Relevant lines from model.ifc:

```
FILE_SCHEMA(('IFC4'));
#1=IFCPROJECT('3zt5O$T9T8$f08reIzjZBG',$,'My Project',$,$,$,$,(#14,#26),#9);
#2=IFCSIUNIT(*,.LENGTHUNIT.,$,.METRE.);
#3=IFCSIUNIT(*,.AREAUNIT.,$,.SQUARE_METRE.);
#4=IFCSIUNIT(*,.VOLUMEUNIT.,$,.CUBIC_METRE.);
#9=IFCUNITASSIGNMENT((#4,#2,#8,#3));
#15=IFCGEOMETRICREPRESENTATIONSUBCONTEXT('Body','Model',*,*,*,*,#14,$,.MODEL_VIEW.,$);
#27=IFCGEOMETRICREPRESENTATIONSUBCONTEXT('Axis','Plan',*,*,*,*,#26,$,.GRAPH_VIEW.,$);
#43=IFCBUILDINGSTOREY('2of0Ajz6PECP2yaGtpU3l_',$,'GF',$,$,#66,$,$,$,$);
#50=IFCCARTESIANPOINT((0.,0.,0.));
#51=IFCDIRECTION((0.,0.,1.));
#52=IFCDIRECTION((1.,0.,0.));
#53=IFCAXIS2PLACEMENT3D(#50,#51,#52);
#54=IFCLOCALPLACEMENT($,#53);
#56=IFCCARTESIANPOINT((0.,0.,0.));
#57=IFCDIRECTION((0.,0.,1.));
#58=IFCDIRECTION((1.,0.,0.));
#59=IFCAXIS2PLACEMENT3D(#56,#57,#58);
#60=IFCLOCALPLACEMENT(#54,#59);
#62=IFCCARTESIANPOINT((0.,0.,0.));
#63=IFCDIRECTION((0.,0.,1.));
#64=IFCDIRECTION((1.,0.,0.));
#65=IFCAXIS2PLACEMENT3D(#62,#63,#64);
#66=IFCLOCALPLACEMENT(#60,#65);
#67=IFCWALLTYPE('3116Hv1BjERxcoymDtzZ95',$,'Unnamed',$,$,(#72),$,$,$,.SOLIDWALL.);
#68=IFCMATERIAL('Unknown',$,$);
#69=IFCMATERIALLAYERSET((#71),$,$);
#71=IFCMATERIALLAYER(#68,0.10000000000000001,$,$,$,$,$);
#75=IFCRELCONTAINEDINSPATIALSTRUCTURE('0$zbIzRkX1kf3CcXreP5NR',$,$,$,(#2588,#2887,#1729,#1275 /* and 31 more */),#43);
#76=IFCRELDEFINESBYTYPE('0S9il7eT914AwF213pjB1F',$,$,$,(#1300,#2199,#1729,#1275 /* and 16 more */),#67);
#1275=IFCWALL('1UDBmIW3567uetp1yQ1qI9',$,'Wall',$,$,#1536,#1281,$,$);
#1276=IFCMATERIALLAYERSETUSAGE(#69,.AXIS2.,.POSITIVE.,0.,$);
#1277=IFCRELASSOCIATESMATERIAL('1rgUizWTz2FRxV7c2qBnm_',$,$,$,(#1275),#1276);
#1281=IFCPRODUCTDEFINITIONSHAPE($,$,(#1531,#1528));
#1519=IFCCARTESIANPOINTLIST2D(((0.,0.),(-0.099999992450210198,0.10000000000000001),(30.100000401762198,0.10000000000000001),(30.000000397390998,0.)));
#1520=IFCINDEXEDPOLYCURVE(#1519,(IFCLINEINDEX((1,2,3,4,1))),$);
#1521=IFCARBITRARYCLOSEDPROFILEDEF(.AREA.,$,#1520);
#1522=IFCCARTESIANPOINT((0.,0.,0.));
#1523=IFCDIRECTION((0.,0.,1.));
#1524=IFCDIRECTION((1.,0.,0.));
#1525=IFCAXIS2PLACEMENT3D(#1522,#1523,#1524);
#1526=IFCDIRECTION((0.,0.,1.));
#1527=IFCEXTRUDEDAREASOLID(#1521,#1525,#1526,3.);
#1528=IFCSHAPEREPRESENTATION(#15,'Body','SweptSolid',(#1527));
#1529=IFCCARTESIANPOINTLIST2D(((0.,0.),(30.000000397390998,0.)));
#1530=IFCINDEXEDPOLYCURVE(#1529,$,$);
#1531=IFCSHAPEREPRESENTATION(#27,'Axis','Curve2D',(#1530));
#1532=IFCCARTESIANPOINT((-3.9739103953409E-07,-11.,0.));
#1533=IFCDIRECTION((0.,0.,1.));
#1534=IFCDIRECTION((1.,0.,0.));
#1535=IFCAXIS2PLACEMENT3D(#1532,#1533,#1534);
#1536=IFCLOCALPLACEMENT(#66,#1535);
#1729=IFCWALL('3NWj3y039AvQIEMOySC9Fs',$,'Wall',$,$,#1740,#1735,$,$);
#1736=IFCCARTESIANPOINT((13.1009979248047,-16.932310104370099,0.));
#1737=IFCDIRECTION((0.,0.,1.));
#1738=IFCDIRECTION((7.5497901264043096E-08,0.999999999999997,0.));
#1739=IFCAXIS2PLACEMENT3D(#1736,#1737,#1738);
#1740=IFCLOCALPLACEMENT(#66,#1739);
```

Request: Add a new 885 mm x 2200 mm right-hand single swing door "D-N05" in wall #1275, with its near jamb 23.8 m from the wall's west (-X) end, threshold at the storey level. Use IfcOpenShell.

```python
import numpy as np
import ifcopenshell
import ifcopenshell.api.feature
import ifcopenshell.api.geometry
import ifcopenshell.api.root
import ifcopenshell.api.spatial
import ifcopenshell.geom
import ifcopenshell.util.element
import ifcopenshell.util.placement
import ifcopenshell.util.representation
import ifcopenshell.util.shape
import ifcopenshell.util.unit

model = ifcopenshell.open("model.ifc")
unit_scale = ifcopenshell.util.unit.calculate_unit_scale(model)
settings = ifcopenshell.geom.settings()


def volume(element):
    """Net volume in cubic metres, openings subtracted."""
    shape = ifcopenshell.geom.create_shape(settings, element)
    return ifcopenshell.util.shape.get_volume(shape.geometry)


wall = model.by_id(1275)
storey = ifcopenshell.util.element.get_container(wall, ifc_class="IfcBuildingStorey")
context = ifcopenshell.util.representation.get_context(model, "Model", "Body", "MODEL_VIEW")
before = volume(wall)

width, height, from_end, sill = 0.885, 2.2, 23.8, 0.0  # metres

# The wall runs along its own X axis, and the end named is its -X end.
wall_shape = ifcopenshell.geom.create_shape(settings, wall)
x, y, z = ifcopenshell.util.shape.get_vertices(wall_shape.geometry).T
start = x.min() + from_end
face, thickness = float(y.min()), float(y.max() - y.min())
wall_matrix = ifcopenshell.util.placement.get_local_placement(wall.ObjectPlacement)
level = ifcopenshell.util.placement.get_local_placement(storey.ObjectPlacement)[2, 3]


def in_wall(x, y):
    """Placement at x, y metres in the wall's axes, at sill height."""
    matrix = wall_matrix.copy()
    matrix[:, 3] = wall_matrix @ np.array([x / unit_scale, y / unit_scale, 0.0, 1.0])
    matrix[2, 3] = level + sill / unit_scale
    return matrix


# Opening: a box that overshoots both wall faces by 50 mm.
opening = ifcopenshell.api.root.create_entity(model, ifc_class="IfcOpeningElement", predefined_type="OPENING")
box = ifcopenshell.api.geometry.add_wall_representation(
    model, context=context, length=width, height=height, thickness=thickness + 0.1
)
ifcopenshell.api.geometry.assign_representation(model, product=opening, representation=box)
ifcopenshell.api.geometry.edit_object_placement(model, product=opening, matrix=in_wall(start, face - 0.05), is_si=False)
ifcopenshell.api.feature.add_feature(model, feature=opening, element=wall)

door = ifcopenshell.api.root.create_entity(model, ifc_class="IfcDoor", name="D-N05", predefined_type="DOOR")
door.OverallWidth, door.OverallHeight = width / unit_scale, height / unit_scale
door.OperationType = "SINGLE_SWING_RIGHT"
body = ifcopenshell.api.geometry.add_door_representation(
    model,
    context=context,
    overall_width=door.OverallWidth,
    overall_height=door.OverallHeight,
    operation_type="SINGLE_SWING_RIGHT",
    lining_properties={"LiningDepth": thickness / unit_scale, "ThresholdDepth": thickness / unit_scale},
)
ifcopenshell.api.geometry.assign_representation(model, product=door, representation=body)
ifcopenshell.api.spatial.assign_container(model, products=[door], relating_structure=storey)
ifcopenshell.api.feature.add_filling(model, opening=opening, element=door)

# The lining spans the wall, so the door starts at the wall face.
ifcopenshell.api.geometry.edit_object_placement(model, product=door, matrix=in_wall(start, face), is_si=False)

after = volume(wall)

print(f"wall volume {before:.3f} -> {after:.3f} m3")

model.write("model_updated.ifc")
```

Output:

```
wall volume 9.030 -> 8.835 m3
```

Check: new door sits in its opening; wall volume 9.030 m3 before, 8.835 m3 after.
